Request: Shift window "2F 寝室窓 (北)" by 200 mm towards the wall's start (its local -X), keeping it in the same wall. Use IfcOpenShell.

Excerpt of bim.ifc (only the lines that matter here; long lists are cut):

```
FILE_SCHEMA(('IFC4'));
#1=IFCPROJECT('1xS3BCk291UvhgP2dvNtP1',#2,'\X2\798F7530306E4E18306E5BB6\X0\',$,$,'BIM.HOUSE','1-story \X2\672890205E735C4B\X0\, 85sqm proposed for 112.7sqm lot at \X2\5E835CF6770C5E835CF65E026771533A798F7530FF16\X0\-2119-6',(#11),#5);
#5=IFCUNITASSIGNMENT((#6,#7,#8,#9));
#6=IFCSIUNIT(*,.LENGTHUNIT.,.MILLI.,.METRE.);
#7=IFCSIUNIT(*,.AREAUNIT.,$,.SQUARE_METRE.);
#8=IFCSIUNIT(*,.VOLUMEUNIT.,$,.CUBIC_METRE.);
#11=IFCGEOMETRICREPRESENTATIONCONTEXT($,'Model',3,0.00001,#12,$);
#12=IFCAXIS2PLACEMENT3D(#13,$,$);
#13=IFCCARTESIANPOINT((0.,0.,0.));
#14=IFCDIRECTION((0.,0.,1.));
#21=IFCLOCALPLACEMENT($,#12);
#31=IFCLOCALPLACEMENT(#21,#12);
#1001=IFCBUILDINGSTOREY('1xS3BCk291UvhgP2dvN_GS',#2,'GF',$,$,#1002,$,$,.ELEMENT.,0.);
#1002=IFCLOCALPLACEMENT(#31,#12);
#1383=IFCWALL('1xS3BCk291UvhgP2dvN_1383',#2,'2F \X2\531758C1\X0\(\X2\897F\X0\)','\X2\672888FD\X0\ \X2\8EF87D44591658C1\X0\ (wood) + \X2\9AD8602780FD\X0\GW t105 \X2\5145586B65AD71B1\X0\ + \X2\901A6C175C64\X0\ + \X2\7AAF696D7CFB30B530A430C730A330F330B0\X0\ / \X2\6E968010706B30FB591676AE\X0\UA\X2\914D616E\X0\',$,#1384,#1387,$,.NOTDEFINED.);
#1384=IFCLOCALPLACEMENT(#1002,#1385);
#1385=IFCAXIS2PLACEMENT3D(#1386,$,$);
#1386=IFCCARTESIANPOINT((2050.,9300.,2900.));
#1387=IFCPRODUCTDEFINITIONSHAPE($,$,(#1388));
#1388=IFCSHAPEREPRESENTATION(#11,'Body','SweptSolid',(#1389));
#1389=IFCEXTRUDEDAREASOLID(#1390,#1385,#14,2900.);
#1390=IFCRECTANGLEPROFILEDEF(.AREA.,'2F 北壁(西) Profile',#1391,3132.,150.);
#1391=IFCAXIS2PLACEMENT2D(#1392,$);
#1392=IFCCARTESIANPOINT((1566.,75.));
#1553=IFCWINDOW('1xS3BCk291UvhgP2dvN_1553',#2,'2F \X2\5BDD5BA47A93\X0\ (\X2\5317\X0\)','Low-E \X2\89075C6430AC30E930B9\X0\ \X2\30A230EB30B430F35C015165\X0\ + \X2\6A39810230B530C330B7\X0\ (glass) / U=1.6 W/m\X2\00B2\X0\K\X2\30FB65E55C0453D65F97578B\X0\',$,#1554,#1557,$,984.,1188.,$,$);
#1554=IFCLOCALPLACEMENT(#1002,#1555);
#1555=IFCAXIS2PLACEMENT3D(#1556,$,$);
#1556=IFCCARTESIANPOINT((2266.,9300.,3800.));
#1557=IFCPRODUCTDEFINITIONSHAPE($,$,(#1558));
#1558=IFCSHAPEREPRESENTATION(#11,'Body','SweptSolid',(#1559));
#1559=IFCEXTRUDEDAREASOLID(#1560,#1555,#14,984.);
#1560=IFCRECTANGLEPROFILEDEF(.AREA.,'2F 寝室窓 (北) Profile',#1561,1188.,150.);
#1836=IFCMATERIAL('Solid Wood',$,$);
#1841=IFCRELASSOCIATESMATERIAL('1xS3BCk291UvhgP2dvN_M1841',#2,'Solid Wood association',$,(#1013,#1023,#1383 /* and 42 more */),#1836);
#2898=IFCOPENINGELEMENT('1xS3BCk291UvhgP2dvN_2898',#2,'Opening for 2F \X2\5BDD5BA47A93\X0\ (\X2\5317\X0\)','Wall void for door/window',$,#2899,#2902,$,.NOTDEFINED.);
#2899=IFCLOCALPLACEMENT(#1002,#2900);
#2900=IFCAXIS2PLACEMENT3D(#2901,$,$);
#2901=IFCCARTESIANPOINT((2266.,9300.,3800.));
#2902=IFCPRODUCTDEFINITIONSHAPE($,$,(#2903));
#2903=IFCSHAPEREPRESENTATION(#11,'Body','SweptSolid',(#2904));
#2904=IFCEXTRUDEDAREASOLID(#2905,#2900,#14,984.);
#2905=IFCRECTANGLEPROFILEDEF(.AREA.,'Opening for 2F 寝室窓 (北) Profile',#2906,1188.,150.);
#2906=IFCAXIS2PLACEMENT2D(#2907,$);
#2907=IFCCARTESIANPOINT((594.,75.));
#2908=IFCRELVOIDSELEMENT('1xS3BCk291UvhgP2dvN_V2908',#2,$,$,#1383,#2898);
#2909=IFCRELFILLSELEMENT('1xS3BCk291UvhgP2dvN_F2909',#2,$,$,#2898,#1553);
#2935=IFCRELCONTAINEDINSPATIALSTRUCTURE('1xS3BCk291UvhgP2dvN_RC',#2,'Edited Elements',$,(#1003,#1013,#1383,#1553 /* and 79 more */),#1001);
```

```python
import ifcopenshell
import ifcopenshell.api.geometry
import ifcopenshell.util.placement

model = ifcopenshell.open("bim.ifc")

window = model.by_guid("1xS3BCk291UvhgP2dvN_1553")
opening = window.FillsVoids[0].RelatingOpeningElement
wall = opening.VoidsElements[0].RelatingBuildingElement

wall_matrix = ifcopenshell.util.placement.get_local_placement(wall.ObjectPlacement)
shift = wall_matrix[:3, 0] * -200.0
before = ifcopenshell.util.placement.get_local_placement(window.ObjectPlacement)[:3, 3].copy()

# The window is not placed relative to its opening, so move both.
for product in (opening, window):
    matrix = ifcopenshell.util.placement.get_local_placement(product.ObjectPlacement)
    matrix[:3, 3] += shift
    ifcopenshell.api.geometry.edit_object_placement(model, product=product, matrix=matrix, is_si=False)

after = ifcopenshell.util.placement.get_local_placement(window.ObjectPlacement)[:3, 3]
print("window moved by", (after - before).round(3) + 0.0)

model.write("bim_updated.ifc")
```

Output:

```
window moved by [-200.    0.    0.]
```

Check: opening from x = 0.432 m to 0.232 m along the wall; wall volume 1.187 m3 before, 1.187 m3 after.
